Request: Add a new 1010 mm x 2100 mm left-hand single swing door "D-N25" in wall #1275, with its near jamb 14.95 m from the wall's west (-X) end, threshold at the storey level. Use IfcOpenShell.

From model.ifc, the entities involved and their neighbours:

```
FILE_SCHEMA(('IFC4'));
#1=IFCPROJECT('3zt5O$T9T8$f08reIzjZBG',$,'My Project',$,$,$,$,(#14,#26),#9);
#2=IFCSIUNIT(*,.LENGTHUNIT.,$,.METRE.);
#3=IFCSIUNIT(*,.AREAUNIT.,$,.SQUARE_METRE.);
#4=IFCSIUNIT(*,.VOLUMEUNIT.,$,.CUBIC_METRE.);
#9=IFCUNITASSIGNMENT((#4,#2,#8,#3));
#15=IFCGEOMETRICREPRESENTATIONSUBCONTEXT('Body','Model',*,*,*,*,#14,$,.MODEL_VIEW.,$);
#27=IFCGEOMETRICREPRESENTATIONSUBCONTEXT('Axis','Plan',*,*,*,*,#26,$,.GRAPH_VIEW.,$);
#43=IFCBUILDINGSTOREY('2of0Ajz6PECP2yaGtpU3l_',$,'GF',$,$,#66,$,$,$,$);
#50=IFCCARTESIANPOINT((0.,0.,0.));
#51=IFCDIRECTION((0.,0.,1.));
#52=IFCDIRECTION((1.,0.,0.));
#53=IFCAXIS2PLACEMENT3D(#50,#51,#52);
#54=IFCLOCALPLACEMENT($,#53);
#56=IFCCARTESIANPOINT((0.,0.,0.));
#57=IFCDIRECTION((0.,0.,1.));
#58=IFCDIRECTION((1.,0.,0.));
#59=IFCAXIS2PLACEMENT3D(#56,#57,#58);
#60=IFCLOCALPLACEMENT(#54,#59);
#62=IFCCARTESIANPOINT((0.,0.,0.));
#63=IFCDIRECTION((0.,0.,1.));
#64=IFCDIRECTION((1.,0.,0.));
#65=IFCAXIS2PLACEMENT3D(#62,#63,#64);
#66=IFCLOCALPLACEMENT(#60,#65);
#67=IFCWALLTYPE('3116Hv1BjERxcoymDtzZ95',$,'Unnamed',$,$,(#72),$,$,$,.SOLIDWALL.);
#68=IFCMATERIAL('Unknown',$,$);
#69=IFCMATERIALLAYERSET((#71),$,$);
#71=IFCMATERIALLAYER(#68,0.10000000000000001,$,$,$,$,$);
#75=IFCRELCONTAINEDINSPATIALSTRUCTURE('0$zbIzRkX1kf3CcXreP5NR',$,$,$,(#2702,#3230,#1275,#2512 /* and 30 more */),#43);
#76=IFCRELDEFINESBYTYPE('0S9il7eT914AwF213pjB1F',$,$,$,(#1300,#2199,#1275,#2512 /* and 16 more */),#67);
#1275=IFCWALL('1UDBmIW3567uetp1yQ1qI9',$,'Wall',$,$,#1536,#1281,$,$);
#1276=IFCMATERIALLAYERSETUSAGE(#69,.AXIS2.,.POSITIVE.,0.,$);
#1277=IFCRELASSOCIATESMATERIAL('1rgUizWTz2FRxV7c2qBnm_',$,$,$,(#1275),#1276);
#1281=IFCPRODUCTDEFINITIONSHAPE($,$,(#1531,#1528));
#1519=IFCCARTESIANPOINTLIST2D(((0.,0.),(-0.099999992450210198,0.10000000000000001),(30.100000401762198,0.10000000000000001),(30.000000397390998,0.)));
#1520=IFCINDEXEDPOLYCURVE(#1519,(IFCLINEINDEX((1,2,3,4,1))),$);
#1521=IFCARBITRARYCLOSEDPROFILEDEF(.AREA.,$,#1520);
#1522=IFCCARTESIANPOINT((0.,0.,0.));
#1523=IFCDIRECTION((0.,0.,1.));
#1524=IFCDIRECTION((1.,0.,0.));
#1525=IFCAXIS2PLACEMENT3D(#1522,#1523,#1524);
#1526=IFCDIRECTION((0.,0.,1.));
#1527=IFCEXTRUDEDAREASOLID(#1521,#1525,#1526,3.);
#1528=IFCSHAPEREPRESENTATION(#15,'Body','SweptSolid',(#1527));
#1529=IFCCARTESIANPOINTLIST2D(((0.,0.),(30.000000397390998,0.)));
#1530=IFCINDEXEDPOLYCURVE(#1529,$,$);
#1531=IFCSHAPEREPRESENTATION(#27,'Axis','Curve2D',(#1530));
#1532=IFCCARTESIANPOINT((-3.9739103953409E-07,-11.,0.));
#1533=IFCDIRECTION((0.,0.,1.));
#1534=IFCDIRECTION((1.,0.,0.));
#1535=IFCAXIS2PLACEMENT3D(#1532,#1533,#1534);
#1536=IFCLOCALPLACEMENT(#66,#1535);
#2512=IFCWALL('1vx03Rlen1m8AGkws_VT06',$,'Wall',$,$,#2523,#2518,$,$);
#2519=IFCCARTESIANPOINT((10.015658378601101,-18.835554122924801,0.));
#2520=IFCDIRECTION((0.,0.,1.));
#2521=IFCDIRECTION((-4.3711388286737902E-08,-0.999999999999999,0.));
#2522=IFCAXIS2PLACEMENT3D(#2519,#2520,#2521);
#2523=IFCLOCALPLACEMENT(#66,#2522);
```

```python
import numpy as np
import ifcopenshell
import ifcopenshell.api.feature
import ifcopenshell.api.geometry
import ifcopenshell.api.root
import ifcopenshell.api.spatial
import ifcopenshell.geom
import ifcopenshell.util.element
import ifcopenshell.util.placement
import ifcopenshell.util.representation
import ifcopenshell.util.shape
import ifcopenshell.util.unit

model = ifcopenshell.open("model.ifc")
unit_scale = ifcopenshell.util.unit.calculate_unit_scale(model)
settings = ifcopenshell.geom.settings()


def volume(element):
    """Net volume in cubic metres, openings subtracted."""
    shape = ifcopenshell.geom.create_shape(settings, element)
    return ifcopenshell.util.shape.get_volume(shape.geometry)


wall = model.by_guid("1UDBmIW3567uetp1yQ1qI9")
storey = ifcopenshell.util.element.get_container(wall, ifc_class="IfcBuildingStorey")
context = ifcopenshell.util.representation.get_context(model, "Model", "Body", "MODEL_VIEW")
before = volume(wall)

width, height, from_end, sill = 1.01, 2.1, 14.95, 0.0  # metres

# The wall runs along its own X axis, and the end named is its -X end.
wall_shape = ifcopenshell.geom.create_shape(settings, wall)
x, y, z = ifcopenshell.util.shape.get_vertices(wall_shape.geometry).T
start = x.min() + from_end
face, thickness = float(y.min()), float(y.max() - y.min())
wall_matrix = ifcopenshell.util.placement.get_local_placement(wall.ObjectPlacement)
level = ifcopenshell.util.placement.get_local_placement(storey.ObjectPlacement)[2, 3]


def in_wall(x, y):
    """Placement at x, y metres in the wall's axes, at sill height."""
    matrix = wall_matrix.copy()
    matrix[:, 3] = wall_matrix @ np.array([x / unit_scale, y / unit_scale, 0.0, 1.0])
    matrix[2, 3] = level + sill / unit_scale
    return matrix


# Opening: a box that overshoots both wall faces by 50 mm.
opening = ifcopenshell.api.root.create_entity(model, ifc_class="IfcOpeningElement", predefined_type="OPENING")
box = ifcopenshell.api.geometry.add_wall_representation(
    model, context=context, length=width, height=height, thickness=thickness + 0.1
)
ifcopenshell.api.geometry.assign_representation(model, product=opening, representation=box)
ifcopenshell.api.geometry.edit_object_placement(model, product=opening, matrix=in_wall(start, face - 0.05), is_si=False)
ifcopenshell.api.feature.add_feature(model, feature=opening, element=wall)

door = ifcopenshell.api.root.create_entity(model, ifc_class="IfcDoor", name="D-N25", predefined_type="DOOR")
door.OverallWidth, door.OverallHeight = width / unit_scale, height / unit_scale
door.OperationType = "SINGLE_SWING_LEFT"
body = ifcopenshell.api.geometry.add_door_representation(
    model,
    context=context,
    overall_width=door.OverallWidth,
    overall_height=door.OverallHeight,
    operation_type="SINGLE_SWING_LEFT",
    lining_properties={"LiningDepth": thickness / unit_scale, "ThresholdDepth": thickness / unit_scale},
)
ifcopenshell.api.geometry.assign_representation(model, product=door, representation=body)
ifcopenshell.api.spatial.assign_container(model, products=[door], relating_structure=storey)
ifcopenshell.api.feature.add_filling(model, opening=opening, element=door)

# The lining spans the wall, so the door starts at the wall face.
ifcopenshell.api.geometry.edit_object_placement(model, product=door, matrix=in_wall(start, face), is_si=False)

after = volume(wall)

print(f"wall volume {before:.3f} -> {after:.3f} m3")

model.write("model_rev.ifc")
```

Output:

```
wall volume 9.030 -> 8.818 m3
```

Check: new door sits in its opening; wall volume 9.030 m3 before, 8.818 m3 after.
